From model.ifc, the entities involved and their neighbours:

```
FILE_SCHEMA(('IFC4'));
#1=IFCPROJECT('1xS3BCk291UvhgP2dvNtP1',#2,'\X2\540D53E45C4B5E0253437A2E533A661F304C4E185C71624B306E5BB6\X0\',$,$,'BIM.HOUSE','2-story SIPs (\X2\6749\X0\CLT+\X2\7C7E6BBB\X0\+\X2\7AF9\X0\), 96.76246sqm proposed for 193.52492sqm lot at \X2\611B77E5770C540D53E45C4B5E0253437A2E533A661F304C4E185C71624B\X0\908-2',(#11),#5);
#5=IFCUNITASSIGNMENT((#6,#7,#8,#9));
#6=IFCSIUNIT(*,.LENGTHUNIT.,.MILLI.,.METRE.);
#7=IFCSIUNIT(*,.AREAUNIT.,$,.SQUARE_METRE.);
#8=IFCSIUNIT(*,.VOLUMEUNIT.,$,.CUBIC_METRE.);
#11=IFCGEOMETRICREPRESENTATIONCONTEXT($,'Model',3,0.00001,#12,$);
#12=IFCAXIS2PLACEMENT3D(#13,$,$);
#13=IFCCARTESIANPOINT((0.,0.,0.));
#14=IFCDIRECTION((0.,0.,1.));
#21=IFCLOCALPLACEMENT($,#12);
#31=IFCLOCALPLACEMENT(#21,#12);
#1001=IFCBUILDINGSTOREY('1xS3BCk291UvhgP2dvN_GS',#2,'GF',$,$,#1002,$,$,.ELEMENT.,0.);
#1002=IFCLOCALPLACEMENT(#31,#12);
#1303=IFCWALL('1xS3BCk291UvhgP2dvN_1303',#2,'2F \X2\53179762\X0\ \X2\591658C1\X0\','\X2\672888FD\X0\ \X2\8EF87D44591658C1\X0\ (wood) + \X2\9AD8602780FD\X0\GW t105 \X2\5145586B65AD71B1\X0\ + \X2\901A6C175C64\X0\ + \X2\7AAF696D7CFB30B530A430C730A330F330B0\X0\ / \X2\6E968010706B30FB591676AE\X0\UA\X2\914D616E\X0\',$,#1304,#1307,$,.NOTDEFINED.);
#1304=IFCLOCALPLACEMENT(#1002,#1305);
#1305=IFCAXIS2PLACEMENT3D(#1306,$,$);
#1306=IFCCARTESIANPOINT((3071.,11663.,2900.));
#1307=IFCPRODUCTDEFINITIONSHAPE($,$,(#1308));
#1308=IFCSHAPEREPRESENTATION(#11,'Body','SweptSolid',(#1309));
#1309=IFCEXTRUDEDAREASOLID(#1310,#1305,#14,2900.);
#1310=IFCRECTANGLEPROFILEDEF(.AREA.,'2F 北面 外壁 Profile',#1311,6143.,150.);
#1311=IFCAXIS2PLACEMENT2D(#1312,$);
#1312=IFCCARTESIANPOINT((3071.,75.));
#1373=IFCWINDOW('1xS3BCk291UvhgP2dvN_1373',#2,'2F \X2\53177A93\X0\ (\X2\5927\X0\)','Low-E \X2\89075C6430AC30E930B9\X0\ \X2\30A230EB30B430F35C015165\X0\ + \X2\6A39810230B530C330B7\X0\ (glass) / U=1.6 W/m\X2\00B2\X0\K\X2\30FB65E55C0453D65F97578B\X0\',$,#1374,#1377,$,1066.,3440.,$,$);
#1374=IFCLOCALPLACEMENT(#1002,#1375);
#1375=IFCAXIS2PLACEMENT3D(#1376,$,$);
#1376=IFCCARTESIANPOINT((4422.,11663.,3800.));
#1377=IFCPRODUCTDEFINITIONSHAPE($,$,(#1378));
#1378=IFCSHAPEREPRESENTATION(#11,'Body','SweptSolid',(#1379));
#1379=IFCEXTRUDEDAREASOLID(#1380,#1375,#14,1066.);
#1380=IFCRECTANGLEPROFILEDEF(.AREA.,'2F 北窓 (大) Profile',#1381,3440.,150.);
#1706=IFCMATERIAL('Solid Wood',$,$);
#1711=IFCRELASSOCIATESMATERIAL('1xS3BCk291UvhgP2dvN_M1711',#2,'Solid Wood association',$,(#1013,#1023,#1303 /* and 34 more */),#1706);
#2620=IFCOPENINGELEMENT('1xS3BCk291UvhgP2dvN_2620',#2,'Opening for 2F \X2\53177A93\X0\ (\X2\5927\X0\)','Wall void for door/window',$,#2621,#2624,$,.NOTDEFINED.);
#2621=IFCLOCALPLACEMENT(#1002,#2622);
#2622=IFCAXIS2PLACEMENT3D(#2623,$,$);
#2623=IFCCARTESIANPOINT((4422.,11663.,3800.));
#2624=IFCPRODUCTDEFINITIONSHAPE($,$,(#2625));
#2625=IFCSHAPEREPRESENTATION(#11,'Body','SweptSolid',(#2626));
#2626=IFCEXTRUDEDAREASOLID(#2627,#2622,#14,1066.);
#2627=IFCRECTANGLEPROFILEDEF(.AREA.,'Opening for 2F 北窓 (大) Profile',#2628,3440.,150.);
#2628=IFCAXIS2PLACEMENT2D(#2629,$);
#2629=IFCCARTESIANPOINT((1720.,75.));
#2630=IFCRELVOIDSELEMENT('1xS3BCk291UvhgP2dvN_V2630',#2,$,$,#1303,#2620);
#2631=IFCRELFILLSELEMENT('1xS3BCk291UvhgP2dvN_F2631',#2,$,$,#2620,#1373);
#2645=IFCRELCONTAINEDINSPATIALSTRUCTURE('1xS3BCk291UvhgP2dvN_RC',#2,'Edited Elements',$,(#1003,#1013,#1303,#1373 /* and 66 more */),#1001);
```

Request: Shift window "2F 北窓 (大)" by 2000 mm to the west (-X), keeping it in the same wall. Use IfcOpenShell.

```python
import ifcopenshell
import ifcopenshell.api.geometry
import ifcopenshell.util.placement

model = ifcopenshell.open("model.ifc")

window = model.by_guid("1xS3BCk291UvhgP2dvN_1373")
opening = window.FillsVoids[0].RelatingOpeningElement
wall = opening.VoidsElements[0].RelatingBuildingElement

wall_matrix = ifcopenshell.util.placement.get_local_placement(wall.ObjectPlacement)
shift = wall_matrix[:3, 0] * -2000.0
before = ifcopenshell.util.placement.get_local_placement(window.ObjectPlacement)[:3, 3].copy()

# The window is not placed relative to its opening, so move both.
for product in (opening, window):
    matrix = ifcopenshell.util.placement.get_local_placement(product.ObjectPlacement)
    matrix[:3, 3] += shift
    ifcopenshell.api.geometry.edit_object_placement(model, product=product, matrix=matrix, is_si=False)

after = ifcopenshell.util.placement.get_local_placement(window.ObjectPlacement)[:3, 3]
print("window moved by", (after - before).round(3) + 0.0)

model.write("model_rev.ifc")
```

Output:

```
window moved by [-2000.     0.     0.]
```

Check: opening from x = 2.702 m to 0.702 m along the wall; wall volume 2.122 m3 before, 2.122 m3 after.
